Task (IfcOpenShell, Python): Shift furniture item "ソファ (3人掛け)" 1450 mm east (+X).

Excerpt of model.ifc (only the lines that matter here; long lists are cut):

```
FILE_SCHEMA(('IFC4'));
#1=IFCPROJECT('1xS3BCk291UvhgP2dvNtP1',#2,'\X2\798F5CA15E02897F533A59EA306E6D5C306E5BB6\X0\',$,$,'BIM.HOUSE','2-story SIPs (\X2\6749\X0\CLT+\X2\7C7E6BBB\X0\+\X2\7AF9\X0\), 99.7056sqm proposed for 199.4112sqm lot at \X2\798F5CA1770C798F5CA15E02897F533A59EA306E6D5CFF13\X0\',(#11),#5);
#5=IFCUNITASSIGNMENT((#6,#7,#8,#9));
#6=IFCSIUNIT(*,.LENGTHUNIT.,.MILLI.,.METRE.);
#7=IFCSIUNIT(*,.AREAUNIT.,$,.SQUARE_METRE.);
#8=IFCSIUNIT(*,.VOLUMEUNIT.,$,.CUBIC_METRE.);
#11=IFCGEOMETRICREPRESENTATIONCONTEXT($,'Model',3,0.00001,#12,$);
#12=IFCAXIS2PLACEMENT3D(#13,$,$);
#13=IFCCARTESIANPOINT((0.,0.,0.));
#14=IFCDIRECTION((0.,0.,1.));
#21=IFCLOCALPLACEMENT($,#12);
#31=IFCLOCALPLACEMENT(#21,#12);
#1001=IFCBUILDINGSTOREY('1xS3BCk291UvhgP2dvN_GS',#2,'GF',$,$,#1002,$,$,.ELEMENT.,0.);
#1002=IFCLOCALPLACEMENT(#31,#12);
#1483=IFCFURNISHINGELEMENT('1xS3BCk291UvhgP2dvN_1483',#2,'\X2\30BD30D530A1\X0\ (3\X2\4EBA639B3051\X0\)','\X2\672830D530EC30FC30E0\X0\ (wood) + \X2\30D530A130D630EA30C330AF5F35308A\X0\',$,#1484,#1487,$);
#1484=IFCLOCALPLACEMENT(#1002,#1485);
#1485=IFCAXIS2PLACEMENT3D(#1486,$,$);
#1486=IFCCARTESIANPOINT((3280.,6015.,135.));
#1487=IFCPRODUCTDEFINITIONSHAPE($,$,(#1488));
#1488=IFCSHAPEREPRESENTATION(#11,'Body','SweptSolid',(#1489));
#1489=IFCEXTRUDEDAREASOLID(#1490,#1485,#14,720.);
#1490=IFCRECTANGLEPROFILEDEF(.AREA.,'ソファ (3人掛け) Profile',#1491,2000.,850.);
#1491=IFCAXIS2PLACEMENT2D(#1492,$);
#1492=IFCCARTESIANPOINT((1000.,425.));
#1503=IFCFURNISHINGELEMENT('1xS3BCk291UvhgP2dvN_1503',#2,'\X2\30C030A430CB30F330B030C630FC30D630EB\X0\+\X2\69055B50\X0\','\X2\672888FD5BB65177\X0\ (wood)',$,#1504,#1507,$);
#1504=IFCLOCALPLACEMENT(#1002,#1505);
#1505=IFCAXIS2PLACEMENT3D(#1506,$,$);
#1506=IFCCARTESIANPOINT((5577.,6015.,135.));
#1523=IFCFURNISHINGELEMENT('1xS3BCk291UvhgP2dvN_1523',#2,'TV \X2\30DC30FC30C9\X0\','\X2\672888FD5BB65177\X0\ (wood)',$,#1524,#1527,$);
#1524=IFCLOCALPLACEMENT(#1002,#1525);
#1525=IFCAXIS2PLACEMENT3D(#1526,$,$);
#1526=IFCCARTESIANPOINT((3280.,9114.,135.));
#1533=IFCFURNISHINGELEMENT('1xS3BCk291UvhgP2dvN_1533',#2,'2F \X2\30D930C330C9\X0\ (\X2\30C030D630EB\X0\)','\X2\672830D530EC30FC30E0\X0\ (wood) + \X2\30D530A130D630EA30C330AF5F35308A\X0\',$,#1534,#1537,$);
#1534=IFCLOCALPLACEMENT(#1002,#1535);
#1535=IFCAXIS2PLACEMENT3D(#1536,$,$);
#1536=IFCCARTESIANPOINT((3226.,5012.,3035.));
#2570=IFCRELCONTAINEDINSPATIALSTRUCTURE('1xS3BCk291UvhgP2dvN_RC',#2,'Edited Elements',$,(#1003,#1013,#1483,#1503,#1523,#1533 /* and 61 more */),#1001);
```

```python
import ifcopenshell
import ifcopenshell.api.geometry
import ifcopenshell.util.placement
import ifcopenshell.util.unit

model = ifcopenshell.open("model.ifc")
unit_scale = ifcopenshell.util.unit.calculate_unit_scale(model)

item = model.by_guid("1xS3BCk291UvhgP2dvN_1483")
matrix = ifcopenshell.util.placement.get_local_placement(item.ObjectPlacement)
matrix[0, 3] += 1.45 / unit_scale
ifcopenshell.api.geometry.edit_object_placement(model, product=item, matrix=matrix, is_si=False)

print(ifcopenshell.util.placement.get_local_placement(item.ObjectPlacement).round(3) + 0.0)

model.write("model_v2.ifc")
```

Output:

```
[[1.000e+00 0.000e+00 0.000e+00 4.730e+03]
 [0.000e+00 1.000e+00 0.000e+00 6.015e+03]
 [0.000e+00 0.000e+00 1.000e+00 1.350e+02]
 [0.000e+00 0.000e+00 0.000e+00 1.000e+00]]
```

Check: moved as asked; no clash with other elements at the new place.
